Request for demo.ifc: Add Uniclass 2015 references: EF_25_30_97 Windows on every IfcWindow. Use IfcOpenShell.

First a look at what the model holds.

```python
import ifcopenshell

model = ifcopenshell.open("demo.ifc")
print(model.schema)
print("classifications:", [c.Name for c in model.by_type("IfcClassification")])
for ifc_class in ("IfcDoor", "IfcRoof", "IfcStair", "IfcWall", "IfcWindow"):
    print(ifc_class, len(model.by_type(ifc_class)))
```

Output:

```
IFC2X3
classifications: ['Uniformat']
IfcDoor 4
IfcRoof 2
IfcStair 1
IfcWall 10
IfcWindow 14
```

```python
import ifcopenshell
import ifcopenshell.api.classification

model = ifcopenshell.open("demo.ifc")

# IFC2X3 requires Source and Edition and has no link from the project to the system.
system = model.create_entity("IfcClassification", Source="NBS", Edition="2015", Name="Uniclass 2015")

codes = {
    "IfcWindow": ("EF_25_30_97", "Windows"),
}
for ifc_class, (code, name) in codes.items():
    products = model.by_type(ifc_class)
    ifcopenshell.api.classification.add_reference(
        model, products=products, classification=system, identification=code, name=name
    )
    print(code, len(products))

model.write("demo-out.ifc")
```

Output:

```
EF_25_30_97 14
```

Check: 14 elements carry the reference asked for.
